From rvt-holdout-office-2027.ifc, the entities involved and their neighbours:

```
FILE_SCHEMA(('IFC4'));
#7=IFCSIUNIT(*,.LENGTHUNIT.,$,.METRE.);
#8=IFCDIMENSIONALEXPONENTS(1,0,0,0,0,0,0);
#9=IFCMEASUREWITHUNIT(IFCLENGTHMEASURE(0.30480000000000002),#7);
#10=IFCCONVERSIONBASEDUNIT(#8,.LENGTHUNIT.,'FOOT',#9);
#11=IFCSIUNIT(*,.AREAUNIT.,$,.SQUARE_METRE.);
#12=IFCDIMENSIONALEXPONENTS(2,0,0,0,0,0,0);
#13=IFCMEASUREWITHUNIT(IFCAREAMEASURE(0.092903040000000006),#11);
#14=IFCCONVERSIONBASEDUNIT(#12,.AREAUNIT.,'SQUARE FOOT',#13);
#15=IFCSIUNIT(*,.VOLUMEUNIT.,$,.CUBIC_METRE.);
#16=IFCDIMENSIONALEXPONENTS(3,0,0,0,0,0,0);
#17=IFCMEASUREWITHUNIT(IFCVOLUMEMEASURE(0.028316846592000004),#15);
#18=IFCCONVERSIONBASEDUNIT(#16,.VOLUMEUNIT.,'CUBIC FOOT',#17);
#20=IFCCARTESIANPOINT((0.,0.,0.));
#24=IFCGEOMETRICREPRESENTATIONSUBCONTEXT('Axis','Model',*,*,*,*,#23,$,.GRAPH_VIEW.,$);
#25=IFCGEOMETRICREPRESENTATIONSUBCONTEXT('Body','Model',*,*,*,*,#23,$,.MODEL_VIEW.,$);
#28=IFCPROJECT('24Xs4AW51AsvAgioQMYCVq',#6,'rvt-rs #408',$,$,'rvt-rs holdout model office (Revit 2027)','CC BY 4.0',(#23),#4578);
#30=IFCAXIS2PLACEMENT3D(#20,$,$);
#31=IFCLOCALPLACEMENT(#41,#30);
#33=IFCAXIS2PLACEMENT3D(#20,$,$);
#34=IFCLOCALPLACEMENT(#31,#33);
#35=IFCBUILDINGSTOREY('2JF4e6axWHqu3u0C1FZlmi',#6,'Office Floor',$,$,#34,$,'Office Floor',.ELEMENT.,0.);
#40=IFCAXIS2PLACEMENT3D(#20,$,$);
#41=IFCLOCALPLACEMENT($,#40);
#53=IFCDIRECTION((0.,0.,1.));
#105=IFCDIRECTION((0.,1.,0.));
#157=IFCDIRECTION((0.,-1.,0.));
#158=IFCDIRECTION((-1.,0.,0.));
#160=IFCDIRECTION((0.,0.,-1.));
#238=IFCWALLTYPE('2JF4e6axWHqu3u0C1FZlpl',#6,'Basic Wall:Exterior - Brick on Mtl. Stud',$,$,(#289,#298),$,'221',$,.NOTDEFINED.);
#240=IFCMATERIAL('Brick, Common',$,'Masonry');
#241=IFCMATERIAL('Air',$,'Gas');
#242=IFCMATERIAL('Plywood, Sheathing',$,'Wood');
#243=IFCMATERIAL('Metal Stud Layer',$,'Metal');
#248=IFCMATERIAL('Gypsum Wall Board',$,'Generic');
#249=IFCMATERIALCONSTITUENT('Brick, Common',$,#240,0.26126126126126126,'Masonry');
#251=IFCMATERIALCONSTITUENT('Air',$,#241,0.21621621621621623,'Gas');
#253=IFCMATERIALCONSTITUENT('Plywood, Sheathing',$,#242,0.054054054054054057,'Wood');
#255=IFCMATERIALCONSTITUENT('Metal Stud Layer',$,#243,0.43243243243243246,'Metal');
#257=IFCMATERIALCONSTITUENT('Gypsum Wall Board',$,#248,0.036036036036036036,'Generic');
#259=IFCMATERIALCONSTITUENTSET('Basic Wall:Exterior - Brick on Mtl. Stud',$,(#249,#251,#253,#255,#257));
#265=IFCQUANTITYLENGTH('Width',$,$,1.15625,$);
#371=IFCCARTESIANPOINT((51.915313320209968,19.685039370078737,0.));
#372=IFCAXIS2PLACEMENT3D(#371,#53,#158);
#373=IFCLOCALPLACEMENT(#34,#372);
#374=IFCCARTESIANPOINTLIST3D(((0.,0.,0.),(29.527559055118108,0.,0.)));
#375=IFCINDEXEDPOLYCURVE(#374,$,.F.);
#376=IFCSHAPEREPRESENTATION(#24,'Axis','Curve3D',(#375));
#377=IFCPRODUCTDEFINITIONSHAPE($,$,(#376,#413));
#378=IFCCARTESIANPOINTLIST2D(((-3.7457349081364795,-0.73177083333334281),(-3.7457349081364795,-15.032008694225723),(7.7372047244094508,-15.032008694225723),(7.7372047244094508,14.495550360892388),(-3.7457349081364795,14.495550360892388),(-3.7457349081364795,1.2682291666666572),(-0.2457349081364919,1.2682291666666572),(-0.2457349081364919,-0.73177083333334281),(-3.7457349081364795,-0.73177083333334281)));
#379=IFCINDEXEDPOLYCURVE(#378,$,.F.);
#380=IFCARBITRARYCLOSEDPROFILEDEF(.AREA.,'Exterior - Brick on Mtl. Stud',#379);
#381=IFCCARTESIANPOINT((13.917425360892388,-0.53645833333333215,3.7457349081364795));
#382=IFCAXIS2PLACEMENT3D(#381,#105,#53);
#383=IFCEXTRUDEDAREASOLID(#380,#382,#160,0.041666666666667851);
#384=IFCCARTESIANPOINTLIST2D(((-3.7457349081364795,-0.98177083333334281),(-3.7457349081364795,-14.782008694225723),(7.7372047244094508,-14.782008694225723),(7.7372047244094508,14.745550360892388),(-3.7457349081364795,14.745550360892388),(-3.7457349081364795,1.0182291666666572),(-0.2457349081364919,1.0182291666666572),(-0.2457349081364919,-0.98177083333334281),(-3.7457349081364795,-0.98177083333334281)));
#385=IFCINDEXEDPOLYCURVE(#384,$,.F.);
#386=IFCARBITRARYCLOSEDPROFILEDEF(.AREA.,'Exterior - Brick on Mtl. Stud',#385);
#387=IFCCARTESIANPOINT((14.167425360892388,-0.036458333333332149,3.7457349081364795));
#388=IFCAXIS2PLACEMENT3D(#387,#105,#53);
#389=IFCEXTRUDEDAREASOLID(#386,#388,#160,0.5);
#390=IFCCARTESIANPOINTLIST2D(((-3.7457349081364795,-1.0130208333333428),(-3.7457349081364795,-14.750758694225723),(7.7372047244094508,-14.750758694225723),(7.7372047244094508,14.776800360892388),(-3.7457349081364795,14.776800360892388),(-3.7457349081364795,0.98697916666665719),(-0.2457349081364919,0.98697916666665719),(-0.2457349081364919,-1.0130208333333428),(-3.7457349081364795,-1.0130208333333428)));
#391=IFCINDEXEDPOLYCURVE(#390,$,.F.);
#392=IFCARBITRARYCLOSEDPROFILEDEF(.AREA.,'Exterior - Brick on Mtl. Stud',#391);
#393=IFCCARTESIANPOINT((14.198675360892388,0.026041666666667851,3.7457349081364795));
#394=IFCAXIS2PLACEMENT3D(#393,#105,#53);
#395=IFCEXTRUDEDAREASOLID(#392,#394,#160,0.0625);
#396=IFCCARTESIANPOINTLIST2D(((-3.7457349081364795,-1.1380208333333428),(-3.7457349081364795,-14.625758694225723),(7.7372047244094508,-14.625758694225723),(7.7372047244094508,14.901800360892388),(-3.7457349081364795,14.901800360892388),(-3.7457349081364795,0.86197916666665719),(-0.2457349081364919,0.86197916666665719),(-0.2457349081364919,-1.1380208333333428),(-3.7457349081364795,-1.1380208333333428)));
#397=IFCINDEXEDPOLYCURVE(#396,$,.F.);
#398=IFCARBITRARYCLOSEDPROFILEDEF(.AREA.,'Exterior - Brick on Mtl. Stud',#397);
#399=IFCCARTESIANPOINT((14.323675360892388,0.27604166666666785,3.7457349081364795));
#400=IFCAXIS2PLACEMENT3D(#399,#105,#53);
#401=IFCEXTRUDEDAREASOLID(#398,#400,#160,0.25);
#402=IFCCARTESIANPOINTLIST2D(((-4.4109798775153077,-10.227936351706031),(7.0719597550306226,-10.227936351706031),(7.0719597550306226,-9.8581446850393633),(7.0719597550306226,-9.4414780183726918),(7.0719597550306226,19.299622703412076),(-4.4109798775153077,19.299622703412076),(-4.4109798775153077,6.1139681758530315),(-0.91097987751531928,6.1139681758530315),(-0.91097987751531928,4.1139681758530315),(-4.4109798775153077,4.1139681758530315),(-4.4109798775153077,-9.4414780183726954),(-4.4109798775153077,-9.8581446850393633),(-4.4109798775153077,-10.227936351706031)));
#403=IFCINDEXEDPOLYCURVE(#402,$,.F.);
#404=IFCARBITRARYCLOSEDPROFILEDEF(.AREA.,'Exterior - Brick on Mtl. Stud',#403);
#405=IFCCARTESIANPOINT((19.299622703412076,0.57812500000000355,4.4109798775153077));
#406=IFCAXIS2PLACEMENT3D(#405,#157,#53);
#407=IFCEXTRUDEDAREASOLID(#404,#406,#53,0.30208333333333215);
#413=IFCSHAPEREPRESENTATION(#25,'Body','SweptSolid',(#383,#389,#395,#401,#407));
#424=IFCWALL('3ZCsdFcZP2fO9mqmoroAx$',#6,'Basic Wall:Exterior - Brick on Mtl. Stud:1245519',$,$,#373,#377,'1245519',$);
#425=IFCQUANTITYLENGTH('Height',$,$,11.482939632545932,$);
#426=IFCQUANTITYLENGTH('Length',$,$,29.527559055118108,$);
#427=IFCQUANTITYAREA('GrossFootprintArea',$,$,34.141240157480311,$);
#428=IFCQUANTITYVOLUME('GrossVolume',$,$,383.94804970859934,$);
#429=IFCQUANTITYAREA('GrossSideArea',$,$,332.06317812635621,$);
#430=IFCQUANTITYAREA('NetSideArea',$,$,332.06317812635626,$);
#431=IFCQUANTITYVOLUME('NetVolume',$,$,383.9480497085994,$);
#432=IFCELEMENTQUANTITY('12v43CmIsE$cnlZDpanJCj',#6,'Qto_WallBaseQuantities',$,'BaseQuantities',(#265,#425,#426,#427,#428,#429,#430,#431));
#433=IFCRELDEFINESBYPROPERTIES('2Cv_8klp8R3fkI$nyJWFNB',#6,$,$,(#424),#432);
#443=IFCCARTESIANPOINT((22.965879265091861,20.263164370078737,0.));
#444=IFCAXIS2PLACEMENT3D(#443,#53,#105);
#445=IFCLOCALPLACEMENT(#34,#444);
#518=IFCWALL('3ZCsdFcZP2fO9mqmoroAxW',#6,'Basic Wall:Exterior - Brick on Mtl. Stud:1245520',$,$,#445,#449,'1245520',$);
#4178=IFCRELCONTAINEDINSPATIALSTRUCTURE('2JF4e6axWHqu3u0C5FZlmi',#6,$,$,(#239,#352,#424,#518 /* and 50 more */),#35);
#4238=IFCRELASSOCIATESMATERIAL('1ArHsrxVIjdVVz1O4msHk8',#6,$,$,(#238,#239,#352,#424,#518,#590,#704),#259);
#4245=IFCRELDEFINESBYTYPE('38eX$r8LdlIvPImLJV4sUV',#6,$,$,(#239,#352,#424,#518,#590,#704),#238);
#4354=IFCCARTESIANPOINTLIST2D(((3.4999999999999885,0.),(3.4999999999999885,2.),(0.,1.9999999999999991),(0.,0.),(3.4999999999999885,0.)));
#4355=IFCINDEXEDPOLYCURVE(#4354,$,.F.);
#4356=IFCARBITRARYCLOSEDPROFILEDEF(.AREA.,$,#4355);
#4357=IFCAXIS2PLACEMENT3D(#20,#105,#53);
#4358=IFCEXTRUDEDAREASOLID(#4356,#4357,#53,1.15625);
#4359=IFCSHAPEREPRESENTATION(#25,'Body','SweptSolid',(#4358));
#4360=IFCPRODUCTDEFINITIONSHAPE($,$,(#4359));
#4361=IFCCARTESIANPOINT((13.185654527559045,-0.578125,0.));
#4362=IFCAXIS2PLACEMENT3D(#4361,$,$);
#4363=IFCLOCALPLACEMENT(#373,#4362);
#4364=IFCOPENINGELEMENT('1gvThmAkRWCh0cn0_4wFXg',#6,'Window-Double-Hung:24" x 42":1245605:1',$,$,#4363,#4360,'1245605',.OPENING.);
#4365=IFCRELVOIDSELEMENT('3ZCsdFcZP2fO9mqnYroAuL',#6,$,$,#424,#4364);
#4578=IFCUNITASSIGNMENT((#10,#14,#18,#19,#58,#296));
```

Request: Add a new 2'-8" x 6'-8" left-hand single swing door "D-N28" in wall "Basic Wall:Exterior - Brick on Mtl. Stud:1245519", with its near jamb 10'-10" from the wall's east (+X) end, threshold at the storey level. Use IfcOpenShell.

```python
import numpy as np
import ifcopenshell
import ifcopenshell.api.feature
import ifcopenshell.api.geometry
import ifcopenshell.api.pset
import ifcopenshell.api.root
import ifcopenshell.api.spatial
import ifcopenshell.geom
import ifcopenshell.util.element
import ifcopenshell.util.placement
import ifcopenshell.util.representation
import ifcopenshell.util.shape
import ifcopenshell.util.unit

model = ifcopenshell.open("rvt-holdout-office-2027.ifc")
unit_scale = ifcopenshell.util.unit.calculate_unit_scale(model)
area_scale = ifcopenshell.util.unit.calculate_unit_scale(model, "AREAUNIT")
volume_scale = ifcopenshell.util.unit.calculate_unit_scale(model, "VOLUMEUNIT")
settings = ifcopenshell.geom.settings()


def volume(element):
    """Net volume in cubic metres, openings subtracted."""
    shape = ifcopenshell.geom.create_shape(settings, element)
    return ifcopenshell.util.shape.get_volume(shape.geometry)


wall = model.by_guid("3ZCsdFcZP2fO9mqmoroAx$")
storey = ifcopenshell.util.element.get_container(wall, ifc_class="IfcBuildingStorey")
context = ifcopenshell.util.representation.get_context(model, "Model", "Body", "MODEL_VIEW")
before = volume(wall)

width, height, from_end, sill = 0.8128, 2.032, 3.302, 0.0  # metres

# The wall runs along its own X axis, and the end named is its -X end.
wall_shape = ifcopenshell.geom.create_shape(settings, wall)
x, y, z = ifcopenshell.util.shape.get_vertices(wall_shape.geometry).T
start = x.min() + from_end
face, thickness = float(y.min()), float(y.max() - y.min())
wall_matrix = ifcopenshell.util.placement.get_local_placement(wall.ObjectPlacement)
level = ifcopenshell.util.placement.get_local_placement(storey.ObjectPlacement)[2, 3]


def in_wall(x, y):
    """Placement at x, y metres in the wall's axes, at sill height."""
    matrix = wall_matrix.copy()
    matrix[:, 3] = wall_matrix @ np.array([x / unit_scale, y / unit_scale, 0.0, 1.0])
    matrix[2, 3] = level + sill / unit_scale
    return matrix


# Opening: a box that overshoots both wall faces by 50 mm.
opening = ifcopenshell.api.root.create_entity(model, ifc_class="IfcOpeningElement", predefined_type="OPENING")
box = ifcopenshell.api.geometry.add_wall_representation(
    model, context=context, length=width, height=height, thickness=thickness + 0.1
)
ifcopenshell.api.geometry.assign_representation(model, product=opening, representation=box)
ifcopenshell.api.geometry.edit_object_placement(model, product=opening, matrix=in_wall(start, face - 0.05), is_si=False)
ifcopenshell.api.feature.add_feature(model, feature=opening, element=wall)

door = ifcopenshell.api.root.create_entity(model, ifc_class="IfcDoor", name="D-N28", predefined_type="DOOR")
door.OverallWidth, door.OverallHeight = width / unit_scale, height / unit_scale
door.OperationType = "SINGLE_SWING_LEFT"
body = ifcopenshell.api.geometry.add_door_representation(
    model,
    context=context,
    overall_width=door.OverallWidth,
    overall_height=door.OverallHeight,
    operation_type="SINGLE_SWING_LEFT",
    lining_properties={"LiningDepth": thickness / unit_scale, "ThresholdDepth": thickness / unit_scale},
)
ifcopenshell.api.geometry.assign_representation(model, product=door, representation=body)
ifcopenshell.api.spatial.assign_container(model, products=[door], relating_structure=storey)
ifcopenshell.api.feature.add_filling(model, opening=opening, element=door)

# The lining spans the wall, so the door starts at the wall face.
ifcopenshell.api.geometry.edit_object_placement(model, product=door, matrix=in_wall(start, face), is_si=False)

after = volume(wall)

# Update the wall's stored quantities.
qto = model.by_id(ifcopenshell.util.element.get_pset(wall, "Qto_WallBaseQuantities", should_inherit=False)["id"])
ifcopenshell.api.pset.edit_qto(model, qto=qto, properties={
    "NetSideArea": after / thickness / area_scale,
    "NetVolume": after / volume_scale,
})

print(f"wall volume {before:.3f} -> {after:.3f} m3")

model.write("rvt-holdout-office-2027-out.ifc")
```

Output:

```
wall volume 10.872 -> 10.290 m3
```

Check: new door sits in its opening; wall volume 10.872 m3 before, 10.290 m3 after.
